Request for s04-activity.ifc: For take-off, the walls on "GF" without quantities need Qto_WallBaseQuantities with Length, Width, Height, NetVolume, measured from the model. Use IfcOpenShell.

First a look at what the model holds.

```python
import ifcopenshell
import ifcopenshell.util.element
import ifcopenshell.util.unit

model = ifcopenshell.open("s04-activity.ifc")
print(model.schema)
for unit_type in ("LENGTHUNIT", "AREAUNIT", "VOLUMEUNIT"):
    print(unit_type, ifcopenshell.util.unit.calculate_unit_scale(model, unit_type))
storey = next(s for s in model.by_type("IfcBuildingStorey") if s.Name == "GF")
walls = [e for e in ifcopenshell.util.element.get_decomposition(storey) if e.is_a("IfcWall")]
for e in sorted(walls, key=lambda e: e.id()):
    print(e.id(), e.is_a(), e.Name, list(ifcopenshell.util.element.get_psets(e, qtos_only=True)), sep=" | ")
```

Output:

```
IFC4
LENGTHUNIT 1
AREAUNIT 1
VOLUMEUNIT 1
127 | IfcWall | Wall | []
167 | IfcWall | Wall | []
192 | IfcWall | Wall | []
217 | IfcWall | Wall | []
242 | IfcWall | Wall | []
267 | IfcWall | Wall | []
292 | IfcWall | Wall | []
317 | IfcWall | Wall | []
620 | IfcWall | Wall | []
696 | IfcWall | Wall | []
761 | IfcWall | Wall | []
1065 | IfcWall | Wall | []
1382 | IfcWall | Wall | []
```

```python
import ifcopenshell
import ifcopenshell.api.pset
import ifcopenshell.geom
import ifcopenshell.util.element
import ifcopenshell.util.shape
import ifcopenshell.util.unit

model = ifcopenshell.open("s04-activity.ifc")
unit_scale = ifcopenshell.util.unit.calculate_unit_scale(model)
volume_scale = ifcopenshell.util.unit.calculate_unit_scale(model, "VOLUMEUNIT")
settings = ifcopenshell.geom.settings()

storey = next(s for s in model.by_type("IfcBuildingStorey") if s.Name == "GF")
walls = [e for e in ifcopenshell.util.element.get_decomposition(storey) if e.is_a("IfcWall")]

for e in sorted(walls, key=lambda e: e.id()):
    if ifcopenshell.util.element.get_psets(e, qtos_only=True, should_inherit=False):
        continue
    # Geometry comes back in metres, in the element's own axes.
    shape = ifcopenshell.geom.create_shape(settings, e)
    values = {
        "Length": ifcopenshell.util.shape.get_x(shape.geometry) / unit_scale,
        "Width": ifcopenshell.util.shape.get_y(shape.geometry) / unit_scale,
        "Height": ifcopenshell.util.shape.get_z(shape.geometry) / unit_scale,
        "NetVolume": ifcopenshell.util.shape.get_volume(shape.geometry) / volume_scale,
    }
    qto = ifcopenshell.api.pset.add_qto(model, product=e, name="Qto_WallBaseQuantities")
    ifcopenshell.api.pset.edit_qto(model, qto=qto, properties=values)
    print(e.id(), {k: round(v, 3) for k, v in values.items()})

model.write("s04-activity_updated.ifc")
```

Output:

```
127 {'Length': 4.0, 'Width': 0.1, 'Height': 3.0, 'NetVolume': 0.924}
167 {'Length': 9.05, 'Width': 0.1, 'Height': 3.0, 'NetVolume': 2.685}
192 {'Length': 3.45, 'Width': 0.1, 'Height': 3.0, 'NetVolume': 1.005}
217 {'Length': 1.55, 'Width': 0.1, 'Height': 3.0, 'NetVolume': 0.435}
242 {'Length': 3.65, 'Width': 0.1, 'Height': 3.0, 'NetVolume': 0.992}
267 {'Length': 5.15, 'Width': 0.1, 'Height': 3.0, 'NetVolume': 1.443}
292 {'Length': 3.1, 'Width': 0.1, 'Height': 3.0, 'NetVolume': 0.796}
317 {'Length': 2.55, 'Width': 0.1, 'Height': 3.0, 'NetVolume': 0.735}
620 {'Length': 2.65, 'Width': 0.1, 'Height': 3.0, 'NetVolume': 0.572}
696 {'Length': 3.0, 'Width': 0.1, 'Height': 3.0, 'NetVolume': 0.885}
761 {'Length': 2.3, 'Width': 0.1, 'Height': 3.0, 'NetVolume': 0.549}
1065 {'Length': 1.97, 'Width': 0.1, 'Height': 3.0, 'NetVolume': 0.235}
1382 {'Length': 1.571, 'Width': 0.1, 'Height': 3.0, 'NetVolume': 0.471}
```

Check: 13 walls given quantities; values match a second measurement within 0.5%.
